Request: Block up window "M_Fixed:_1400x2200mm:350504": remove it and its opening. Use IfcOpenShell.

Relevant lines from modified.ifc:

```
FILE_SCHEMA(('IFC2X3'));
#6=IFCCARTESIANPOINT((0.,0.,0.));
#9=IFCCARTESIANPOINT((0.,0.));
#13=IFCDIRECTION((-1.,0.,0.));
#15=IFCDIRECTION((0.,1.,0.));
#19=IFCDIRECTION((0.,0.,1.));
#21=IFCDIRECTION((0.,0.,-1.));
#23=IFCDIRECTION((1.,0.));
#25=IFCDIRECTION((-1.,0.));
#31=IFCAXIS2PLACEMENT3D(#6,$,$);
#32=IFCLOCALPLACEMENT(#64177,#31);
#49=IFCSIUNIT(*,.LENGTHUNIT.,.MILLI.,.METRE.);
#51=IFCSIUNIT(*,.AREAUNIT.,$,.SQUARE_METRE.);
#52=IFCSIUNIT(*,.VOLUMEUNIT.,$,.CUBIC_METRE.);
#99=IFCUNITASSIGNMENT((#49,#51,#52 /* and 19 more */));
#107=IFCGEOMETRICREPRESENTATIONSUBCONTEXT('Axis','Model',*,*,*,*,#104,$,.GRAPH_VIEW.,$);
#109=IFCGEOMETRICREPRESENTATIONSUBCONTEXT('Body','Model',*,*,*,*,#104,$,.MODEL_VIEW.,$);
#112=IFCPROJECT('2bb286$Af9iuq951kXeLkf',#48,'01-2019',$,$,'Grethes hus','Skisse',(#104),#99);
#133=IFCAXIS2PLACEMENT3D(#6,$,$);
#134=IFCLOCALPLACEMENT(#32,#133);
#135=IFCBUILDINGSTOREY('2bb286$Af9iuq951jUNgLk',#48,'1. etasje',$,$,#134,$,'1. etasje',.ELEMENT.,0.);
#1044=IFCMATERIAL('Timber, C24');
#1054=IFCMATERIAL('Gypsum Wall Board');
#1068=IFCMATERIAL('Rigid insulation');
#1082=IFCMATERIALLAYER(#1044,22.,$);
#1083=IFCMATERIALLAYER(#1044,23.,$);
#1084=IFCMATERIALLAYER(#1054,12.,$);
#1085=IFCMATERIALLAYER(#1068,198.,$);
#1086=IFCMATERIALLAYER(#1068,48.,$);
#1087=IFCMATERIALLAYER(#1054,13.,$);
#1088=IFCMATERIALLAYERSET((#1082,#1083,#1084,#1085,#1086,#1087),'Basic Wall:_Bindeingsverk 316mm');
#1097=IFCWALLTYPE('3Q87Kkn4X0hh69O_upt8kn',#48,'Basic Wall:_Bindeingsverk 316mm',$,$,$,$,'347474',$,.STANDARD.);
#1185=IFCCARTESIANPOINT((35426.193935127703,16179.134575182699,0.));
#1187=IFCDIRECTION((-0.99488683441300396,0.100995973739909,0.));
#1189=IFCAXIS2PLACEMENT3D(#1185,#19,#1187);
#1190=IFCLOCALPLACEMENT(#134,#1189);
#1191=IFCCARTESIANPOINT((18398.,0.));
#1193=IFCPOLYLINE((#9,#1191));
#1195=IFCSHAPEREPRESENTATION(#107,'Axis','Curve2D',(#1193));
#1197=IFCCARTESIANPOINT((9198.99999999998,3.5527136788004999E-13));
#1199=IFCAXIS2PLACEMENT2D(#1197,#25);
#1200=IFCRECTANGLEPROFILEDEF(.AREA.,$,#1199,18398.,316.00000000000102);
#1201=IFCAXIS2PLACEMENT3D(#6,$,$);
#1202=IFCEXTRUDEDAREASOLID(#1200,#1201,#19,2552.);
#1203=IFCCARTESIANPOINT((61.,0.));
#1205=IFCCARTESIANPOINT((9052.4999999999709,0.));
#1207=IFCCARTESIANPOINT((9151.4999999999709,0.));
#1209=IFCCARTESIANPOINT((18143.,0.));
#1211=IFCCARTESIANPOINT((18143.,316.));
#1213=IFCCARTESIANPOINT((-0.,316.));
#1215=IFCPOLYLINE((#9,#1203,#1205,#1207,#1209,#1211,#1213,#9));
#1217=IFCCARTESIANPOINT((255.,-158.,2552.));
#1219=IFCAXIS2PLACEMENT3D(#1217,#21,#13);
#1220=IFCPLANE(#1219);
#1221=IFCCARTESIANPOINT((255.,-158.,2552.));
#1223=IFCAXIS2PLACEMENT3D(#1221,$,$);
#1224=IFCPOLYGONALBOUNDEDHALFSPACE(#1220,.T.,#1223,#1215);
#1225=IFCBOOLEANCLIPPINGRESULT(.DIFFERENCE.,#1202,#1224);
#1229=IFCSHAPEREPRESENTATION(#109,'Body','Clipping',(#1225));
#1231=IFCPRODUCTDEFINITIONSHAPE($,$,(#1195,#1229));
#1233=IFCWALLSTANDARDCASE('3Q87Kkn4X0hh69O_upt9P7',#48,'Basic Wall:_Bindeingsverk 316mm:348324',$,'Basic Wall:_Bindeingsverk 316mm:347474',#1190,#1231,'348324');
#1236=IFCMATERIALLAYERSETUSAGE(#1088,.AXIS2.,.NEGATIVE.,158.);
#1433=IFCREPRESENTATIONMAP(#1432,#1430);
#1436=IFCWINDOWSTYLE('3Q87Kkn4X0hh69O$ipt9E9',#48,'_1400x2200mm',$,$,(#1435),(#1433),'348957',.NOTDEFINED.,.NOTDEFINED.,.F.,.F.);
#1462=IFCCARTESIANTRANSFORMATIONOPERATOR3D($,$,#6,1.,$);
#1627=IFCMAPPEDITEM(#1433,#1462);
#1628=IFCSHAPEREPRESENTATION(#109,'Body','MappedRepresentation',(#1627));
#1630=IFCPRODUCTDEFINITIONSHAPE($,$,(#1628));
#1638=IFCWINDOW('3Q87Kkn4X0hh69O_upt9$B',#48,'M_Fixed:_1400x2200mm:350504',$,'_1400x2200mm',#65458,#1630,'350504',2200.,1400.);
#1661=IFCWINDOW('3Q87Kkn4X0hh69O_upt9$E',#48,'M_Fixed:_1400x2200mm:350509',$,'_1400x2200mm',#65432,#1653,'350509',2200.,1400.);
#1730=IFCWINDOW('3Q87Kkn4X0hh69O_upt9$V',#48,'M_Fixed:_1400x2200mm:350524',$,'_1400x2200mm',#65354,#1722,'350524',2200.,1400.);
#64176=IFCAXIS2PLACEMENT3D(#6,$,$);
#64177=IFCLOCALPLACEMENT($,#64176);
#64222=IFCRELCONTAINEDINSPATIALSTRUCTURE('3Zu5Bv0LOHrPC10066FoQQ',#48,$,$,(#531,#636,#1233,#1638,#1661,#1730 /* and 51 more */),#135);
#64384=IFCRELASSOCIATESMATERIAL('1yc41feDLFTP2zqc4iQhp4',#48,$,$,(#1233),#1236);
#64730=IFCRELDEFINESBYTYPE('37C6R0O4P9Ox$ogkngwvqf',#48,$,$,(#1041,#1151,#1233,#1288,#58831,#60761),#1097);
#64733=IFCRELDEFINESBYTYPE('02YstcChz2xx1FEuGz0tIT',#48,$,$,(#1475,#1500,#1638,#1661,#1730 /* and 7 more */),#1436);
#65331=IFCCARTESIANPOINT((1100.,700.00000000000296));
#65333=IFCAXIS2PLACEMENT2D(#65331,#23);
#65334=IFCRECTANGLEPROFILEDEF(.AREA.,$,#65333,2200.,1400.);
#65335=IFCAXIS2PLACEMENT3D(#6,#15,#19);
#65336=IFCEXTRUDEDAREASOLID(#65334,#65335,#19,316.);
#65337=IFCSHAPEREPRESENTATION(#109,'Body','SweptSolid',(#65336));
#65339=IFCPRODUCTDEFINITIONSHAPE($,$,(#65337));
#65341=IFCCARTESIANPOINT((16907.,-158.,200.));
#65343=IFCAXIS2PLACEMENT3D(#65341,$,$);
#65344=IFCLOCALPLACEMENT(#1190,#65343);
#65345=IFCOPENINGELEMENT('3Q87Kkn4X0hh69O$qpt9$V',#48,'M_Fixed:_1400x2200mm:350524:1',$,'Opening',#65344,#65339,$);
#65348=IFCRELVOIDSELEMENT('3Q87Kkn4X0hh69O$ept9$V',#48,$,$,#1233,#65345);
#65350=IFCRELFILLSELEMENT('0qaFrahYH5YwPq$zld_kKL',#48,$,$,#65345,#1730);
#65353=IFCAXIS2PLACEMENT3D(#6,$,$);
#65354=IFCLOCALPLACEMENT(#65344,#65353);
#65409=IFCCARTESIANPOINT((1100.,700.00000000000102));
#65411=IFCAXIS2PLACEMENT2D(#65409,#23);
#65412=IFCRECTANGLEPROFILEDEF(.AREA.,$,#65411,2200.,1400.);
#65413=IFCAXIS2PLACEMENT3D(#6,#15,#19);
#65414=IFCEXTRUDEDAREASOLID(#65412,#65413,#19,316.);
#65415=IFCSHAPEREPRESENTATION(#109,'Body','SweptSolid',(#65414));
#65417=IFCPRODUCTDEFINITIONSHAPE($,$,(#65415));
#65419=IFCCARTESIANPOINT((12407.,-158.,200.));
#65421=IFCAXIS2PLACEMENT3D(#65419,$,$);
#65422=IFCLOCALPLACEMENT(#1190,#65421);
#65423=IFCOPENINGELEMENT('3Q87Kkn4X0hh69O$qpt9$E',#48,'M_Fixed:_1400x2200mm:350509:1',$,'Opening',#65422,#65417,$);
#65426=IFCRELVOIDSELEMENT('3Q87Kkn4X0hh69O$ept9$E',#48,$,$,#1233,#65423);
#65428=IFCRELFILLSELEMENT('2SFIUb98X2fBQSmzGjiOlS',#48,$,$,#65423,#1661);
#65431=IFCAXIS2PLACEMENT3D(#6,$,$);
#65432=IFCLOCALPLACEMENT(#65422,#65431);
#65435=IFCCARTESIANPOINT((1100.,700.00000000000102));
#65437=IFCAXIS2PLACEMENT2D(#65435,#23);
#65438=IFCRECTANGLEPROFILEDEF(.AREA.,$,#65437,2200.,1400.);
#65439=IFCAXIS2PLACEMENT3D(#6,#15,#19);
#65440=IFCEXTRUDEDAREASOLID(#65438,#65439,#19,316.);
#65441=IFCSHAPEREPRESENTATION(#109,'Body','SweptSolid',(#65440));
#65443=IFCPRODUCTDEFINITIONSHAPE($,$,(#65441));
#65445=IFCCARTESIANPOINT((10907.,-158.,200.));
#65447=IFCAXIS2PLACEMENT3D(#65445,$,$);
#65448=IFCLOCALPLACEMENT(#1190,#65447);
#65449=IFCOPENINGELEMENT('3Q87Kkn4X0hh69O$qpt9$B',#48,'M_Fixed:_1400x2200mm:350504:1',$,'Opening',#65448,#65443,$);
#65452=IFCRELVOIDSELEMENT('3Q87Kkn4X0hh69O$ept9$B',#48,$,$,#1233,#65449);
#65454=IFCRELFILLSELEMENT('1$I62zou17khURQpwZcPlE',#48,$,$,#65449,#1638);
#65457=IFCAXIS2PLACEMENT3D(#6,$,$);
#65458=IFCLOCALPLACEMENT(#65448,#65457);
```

```python
import ifcopenshell
import ifcopenshell.api.feature
import ifcopenshell.api.root
import ifcopenshell.geom
import ifcopenshell.util.shape

model = ifcopenshell.open("modified.ifc")
settings = ifcopenshell.geom.settings()


def volume(element):
    """Net volume in cubic metres, openings subtracted."""
    shape = ifcopenshell.geom.create_shape(settings, element)
    return ifcopenshell.util.shape.get_volume(shape.geometry)


window = model.by_guid("3Q87Kkn4X0hh69O_upt9$B")
opening = window.FillsVoids[0].RelatingOpeningElement
wall = opening.VoidsElements[0].RelatingBuildingElement
before = volume(wall)

ifcopenshell.api.root.remove_product(model, product=window)
ifcopenshell.api.feature.remove_feature(model, feature=opening)

after = volume(wall)

print(f"wall volume {before:.3f} -> {after:.3f} m3")

model.write("modified_updated.ifc")
```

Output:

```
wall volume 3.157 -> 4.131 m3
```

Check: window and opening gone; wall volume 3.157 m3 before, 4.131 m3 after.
